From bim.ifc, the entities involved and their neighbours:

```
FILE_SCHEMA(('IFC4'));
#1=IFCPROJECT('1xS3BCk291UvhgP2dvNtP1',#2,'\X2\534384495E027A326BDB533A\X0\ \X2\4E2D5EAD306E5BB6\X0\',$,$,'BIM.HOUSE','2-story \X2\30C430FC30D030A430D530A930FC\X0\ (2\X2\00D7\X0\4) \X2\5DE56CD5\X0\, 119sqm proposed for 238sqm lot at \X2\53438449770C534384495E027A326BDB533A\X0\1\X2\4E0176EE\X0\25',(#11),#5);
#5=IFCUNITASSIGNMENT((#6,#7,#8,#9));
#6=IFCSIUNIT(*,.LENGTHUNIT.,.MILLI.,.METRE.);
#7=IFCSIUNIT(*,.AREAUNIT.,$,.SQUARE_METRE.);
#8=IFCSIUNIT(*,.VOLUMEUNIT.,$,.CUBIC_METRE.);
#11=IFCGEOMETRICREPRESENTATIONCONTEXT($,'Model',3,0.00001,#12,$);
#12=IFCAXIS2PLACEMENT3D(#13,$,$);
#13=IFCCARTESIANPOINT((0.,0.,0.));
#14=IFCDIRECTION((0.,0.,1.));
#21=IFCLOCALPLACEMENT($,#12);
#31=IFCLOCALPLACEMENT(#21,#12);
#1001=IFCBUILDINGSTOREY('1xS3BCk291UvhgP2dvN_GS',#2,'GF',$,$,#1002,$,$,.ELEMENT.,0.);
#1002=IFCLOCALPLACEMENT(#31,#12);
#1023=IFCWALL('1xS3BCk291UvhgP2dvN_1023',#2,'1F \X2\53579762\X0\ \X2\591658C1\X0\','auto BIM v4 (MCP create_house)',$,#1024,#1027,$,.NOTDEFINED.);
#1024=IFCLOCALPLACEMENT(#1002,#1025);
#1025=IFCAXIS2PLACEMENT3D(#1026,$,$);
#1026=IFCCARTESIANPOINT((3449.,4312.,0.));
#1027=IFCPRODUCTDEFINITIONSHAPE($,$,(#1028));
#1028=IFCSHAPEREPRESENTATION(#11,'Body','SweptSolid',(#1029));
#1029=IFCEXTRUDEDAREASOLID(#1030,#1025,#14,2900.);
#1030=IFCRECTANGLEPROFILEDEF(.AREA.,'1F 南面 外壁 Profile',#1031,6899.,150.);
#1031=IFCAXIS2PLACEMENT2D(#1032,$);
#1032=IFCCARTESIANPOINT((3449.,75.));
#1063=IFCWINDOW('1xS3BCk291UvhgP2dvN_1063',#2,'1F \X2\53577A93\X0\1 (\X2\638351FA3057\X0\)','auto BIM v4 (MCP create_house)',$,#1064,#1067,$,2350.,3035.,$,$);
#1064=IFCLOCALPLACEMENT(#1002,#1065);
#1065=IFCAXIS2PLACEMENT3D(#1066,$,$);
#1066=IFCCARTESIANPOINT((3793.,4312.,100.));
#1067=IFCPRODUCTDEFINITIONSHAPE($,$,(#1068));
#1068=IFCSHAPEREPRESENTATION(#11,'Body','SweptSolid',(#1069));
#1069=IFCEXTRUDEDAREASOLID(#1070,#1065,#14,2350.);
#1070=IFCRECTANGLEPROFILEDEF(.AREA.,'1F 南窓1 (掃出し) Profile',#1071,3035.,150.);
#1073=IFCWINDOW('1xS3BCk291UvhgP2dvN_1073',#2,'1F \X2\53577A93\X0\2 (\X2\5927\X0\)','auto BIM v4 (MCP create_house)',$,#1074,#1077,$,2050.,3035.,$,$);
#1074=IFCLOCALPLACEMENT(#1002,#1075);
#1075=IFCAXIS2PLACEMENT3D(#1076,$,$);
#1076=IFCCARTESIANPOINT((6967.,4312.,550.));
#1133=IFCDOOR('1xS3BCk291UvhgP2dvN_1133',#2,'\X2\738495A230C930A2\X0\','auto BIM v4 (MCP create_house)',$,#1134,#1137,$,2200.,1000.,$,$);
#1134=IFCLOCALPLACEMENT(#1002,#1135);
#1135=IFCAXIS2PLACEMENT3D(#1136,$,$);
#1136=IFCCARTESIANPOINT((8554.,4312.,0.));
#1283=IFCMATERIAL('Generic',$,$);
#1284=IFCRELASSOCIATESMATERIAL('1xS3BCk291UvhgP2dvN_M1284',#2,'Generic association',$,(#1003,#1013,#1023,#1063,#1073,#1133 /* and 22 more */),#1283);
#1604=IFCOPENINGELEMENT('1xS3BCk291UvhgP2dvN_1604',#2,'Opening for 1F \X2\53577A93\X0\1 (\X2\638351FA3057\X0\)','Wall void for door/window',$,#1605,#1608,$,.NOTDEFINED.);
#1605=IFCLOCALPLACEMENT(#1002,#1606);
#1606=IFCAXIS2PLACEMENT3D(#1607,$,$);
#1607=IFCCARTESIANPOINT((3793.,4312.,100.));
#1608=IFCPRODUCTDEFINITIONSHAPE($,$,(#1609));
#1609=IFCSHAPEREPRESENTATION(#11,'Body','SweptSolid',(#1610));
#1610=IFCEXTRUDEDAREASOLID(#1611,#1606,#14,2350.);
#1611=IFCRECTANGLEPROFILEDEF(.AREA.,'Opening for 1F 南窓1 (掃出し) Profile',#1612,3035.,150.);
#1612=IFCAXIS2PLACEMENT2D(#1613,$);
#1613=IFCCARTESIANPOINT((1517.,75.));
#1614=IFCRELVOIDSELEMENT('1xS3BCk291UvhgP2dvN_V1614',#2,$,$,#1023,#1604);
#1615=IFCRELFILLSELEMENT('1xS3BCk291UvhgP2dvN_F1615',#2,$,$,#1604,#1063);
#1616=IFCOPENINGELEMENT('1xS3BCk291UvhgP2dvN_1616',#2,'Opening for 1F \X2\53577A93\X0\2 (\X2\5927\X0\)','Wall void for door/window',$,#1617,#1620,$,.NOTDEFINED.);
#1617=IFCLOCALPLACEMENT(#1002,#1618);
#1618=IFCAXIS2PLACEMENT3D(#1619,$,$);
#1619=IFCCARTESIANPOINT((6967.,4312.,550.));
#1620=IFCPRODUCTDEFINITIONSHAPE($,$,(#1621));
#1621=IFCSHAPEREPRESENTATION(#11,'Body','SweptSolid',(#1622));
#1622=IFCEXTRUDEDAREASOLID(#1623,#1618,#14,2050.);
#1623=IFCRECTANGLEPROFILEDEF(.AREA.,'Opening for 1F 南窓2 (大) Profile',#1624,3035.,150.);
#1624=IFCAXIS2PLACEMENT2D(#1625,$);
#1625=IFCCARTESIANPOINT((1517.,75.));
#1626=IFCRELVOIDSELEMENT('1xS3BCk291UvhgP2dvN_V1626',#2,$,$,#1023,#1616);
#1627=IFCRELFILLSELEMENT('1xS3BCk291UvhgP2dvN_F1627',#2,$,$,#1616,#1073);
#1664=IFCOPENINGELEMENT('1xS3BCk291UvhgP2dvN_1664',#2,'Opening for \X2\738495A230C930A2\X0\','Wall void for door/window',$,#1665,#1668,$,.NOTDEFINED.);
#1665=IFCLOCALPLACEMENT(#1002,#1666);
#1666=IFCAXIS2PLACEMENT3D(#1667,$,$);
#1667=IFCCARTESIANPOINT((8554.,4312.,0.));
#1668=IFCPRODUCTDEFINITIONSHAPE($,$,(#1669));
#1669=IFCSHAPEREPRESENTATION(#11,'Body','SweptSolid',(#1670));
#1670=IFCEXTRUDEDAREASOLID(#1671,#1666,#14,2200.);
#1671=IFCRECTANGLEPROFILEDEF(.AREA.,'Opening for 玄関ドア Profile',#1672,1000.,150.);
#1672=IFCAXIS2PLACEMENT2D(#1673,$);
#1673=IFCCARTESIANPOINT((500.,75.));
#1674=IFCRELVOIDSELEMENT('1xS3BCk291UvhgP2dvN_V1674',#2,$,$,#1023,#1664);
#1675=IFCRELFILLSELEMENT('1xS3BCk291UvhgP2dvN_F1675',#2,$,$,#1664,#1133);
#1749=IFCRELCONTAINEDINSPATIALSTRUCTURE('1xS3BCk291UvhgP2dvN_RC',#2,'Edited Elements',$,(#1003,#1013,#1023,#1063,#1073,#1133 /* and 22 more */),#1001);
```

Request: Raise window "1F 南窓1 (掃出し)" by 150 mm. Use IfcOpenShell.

```python
import numpy as np
import ifcopenshell
import ifcopenshell.api.geometry
import ifcopenshell.util.placement
import ifcopenshell.util.unit

model = ifcopenshell.open("bim.ifc")
unit_scale = ifcopenshell.util.unit.calculate_unit_scale(model)

window = model.by_id(1063)
opening = window.FillsVoids[0].RelatingOpeningElement
dz = 0.15 / unit_scale

shift = np.array([0.0, 0.0, dz])
# The window is not placed relative to its opening, so move both.
for product in (opening, window):
    matrix = ifcopenshell.util.placement.get_local_placement(product.ObjectPlacement)
    matrix[:3, 3] += shift
    ifcopenshell.api.geometry.edit_object_placement(model, product=product, matrix=matrix, is_si=False)

print(f"moved by {dz * unit_scale:+.3f} m")

model.write("bim_rev.ifc")
```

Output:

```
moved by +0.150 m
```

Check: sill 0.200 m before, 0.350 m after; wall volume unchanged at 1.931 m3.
